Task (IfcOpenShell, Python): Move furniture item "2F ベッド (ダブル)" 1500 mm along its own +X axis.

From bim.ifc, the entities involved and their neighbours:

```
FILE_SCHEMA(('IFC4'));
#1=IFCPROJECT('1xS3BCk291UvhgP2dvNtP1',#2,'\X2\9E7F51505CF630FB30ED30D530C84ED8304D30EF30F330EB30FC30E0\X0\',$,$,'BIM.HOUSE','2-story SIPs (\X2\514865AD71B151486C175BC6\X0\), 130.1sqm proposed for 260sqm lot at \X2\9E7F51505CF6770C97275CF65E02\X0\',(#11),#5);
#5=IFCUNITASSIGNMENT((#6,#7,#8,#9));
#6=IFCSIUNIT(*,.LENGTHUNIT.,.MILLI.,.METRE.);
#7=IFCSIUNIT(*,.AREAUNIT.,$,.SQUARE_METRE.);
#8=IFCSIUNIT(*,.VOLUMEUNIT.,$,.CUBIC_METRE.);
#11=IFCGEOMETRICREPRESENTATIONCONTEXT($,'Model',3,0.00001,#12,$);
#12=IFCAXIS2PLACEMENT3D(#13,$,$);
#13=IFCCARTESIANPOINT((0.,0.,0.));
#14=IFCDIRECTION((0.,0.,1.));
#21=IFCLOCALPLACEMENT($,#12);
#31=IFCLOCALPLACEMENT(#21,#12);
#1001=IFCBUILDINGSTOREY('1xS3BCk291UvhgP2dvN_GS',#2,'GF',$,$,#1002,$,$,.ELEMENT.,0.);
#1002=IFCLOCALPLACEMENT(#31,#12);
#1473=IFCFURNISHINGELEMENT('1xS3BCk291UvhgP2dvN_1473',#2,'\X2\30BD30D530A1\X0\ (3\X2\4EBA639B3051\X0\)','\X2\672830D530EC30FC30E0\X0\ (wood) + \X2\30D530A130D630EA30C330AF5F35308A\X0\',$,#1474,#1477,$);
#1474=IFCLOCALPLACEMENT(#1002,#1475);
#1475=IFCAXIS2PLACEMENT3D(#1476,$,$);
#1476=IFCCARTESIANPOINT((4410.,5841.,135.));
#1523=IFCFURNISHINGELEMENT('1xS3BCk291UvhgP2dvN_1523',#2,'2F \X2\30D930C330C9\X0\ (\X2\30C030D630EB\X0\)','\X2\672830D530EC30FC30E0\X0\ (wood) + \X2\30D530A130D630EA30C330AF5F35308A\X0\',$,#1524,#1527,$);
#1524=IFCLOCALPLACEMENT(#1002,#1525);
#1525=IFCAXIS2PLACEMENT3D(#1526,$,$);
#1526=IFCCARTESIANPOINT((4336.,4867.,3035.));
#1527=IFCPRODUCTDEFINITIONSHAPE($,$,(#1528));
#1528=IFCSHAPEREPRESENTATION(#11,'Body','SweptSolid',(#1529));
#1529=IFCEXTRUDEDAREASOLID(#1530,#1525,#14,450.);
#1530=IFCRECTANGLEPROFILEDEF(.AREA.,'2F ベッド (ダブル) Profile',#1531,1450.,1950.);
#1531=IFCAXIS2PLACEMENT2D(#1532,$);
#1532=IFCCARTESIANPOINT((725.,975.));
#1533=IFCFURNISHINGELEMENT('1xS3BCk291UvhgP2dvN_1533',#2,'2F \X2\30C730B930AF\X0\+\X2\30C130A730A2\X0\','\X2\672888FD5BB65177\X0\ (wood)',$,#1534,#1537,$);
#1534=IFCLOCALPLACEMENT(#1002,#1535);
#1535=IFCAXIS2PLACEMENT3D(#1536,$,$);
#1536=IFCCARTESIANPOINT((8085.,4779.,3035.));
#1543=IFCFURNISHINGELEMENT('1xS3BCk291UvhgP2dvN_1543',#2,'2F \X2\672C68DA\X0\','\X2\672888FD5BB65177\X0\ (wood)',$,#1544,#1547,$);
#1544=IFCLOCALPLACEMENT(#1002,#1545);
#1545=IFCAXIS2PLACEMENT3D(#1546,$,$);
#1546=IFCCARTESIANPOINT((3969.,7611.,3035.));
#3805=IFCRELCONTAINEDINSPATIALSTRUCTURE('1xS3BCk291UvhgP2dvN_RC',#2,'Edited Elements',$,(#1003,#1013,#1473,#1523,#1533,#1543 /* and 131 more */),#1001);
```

```python
import ifcopenshell
import ifcopenshell.api.geometry
import ifcopenshell.util.placement
import ifcopenshell.util.unit

model = ifcopenshell.open("bim.ifc")
unit_scale = ifcopenshell.util.unit.calculate_unit_scale(model)

item = model.by_guid("1xS3BCk291UvhgP2dvN_1523")
matrix = ifcopenshell.util.placement.get_local_placement(item.ObjectPlacement)
matrix[:3, 3] += matrix[:3, 0] * 1.5 / unit_scale
ifcopenshell.api.geometry.edit_object_placement(model, product=item, matrix=matrix, is_si=False)

print(ifcopenshell.util.placement.get_local_placement(item.ObjectPlacement).round(3) + 0.0)

model.write("bim_rev.ifc")
```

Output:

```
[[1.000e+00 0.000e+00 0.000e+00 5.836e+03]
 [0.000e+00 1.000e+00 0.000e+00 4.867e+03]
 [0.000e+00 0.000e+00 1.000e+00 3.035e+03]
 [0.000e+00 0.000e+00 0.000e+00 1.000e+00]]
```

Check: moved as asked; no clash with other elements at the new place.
